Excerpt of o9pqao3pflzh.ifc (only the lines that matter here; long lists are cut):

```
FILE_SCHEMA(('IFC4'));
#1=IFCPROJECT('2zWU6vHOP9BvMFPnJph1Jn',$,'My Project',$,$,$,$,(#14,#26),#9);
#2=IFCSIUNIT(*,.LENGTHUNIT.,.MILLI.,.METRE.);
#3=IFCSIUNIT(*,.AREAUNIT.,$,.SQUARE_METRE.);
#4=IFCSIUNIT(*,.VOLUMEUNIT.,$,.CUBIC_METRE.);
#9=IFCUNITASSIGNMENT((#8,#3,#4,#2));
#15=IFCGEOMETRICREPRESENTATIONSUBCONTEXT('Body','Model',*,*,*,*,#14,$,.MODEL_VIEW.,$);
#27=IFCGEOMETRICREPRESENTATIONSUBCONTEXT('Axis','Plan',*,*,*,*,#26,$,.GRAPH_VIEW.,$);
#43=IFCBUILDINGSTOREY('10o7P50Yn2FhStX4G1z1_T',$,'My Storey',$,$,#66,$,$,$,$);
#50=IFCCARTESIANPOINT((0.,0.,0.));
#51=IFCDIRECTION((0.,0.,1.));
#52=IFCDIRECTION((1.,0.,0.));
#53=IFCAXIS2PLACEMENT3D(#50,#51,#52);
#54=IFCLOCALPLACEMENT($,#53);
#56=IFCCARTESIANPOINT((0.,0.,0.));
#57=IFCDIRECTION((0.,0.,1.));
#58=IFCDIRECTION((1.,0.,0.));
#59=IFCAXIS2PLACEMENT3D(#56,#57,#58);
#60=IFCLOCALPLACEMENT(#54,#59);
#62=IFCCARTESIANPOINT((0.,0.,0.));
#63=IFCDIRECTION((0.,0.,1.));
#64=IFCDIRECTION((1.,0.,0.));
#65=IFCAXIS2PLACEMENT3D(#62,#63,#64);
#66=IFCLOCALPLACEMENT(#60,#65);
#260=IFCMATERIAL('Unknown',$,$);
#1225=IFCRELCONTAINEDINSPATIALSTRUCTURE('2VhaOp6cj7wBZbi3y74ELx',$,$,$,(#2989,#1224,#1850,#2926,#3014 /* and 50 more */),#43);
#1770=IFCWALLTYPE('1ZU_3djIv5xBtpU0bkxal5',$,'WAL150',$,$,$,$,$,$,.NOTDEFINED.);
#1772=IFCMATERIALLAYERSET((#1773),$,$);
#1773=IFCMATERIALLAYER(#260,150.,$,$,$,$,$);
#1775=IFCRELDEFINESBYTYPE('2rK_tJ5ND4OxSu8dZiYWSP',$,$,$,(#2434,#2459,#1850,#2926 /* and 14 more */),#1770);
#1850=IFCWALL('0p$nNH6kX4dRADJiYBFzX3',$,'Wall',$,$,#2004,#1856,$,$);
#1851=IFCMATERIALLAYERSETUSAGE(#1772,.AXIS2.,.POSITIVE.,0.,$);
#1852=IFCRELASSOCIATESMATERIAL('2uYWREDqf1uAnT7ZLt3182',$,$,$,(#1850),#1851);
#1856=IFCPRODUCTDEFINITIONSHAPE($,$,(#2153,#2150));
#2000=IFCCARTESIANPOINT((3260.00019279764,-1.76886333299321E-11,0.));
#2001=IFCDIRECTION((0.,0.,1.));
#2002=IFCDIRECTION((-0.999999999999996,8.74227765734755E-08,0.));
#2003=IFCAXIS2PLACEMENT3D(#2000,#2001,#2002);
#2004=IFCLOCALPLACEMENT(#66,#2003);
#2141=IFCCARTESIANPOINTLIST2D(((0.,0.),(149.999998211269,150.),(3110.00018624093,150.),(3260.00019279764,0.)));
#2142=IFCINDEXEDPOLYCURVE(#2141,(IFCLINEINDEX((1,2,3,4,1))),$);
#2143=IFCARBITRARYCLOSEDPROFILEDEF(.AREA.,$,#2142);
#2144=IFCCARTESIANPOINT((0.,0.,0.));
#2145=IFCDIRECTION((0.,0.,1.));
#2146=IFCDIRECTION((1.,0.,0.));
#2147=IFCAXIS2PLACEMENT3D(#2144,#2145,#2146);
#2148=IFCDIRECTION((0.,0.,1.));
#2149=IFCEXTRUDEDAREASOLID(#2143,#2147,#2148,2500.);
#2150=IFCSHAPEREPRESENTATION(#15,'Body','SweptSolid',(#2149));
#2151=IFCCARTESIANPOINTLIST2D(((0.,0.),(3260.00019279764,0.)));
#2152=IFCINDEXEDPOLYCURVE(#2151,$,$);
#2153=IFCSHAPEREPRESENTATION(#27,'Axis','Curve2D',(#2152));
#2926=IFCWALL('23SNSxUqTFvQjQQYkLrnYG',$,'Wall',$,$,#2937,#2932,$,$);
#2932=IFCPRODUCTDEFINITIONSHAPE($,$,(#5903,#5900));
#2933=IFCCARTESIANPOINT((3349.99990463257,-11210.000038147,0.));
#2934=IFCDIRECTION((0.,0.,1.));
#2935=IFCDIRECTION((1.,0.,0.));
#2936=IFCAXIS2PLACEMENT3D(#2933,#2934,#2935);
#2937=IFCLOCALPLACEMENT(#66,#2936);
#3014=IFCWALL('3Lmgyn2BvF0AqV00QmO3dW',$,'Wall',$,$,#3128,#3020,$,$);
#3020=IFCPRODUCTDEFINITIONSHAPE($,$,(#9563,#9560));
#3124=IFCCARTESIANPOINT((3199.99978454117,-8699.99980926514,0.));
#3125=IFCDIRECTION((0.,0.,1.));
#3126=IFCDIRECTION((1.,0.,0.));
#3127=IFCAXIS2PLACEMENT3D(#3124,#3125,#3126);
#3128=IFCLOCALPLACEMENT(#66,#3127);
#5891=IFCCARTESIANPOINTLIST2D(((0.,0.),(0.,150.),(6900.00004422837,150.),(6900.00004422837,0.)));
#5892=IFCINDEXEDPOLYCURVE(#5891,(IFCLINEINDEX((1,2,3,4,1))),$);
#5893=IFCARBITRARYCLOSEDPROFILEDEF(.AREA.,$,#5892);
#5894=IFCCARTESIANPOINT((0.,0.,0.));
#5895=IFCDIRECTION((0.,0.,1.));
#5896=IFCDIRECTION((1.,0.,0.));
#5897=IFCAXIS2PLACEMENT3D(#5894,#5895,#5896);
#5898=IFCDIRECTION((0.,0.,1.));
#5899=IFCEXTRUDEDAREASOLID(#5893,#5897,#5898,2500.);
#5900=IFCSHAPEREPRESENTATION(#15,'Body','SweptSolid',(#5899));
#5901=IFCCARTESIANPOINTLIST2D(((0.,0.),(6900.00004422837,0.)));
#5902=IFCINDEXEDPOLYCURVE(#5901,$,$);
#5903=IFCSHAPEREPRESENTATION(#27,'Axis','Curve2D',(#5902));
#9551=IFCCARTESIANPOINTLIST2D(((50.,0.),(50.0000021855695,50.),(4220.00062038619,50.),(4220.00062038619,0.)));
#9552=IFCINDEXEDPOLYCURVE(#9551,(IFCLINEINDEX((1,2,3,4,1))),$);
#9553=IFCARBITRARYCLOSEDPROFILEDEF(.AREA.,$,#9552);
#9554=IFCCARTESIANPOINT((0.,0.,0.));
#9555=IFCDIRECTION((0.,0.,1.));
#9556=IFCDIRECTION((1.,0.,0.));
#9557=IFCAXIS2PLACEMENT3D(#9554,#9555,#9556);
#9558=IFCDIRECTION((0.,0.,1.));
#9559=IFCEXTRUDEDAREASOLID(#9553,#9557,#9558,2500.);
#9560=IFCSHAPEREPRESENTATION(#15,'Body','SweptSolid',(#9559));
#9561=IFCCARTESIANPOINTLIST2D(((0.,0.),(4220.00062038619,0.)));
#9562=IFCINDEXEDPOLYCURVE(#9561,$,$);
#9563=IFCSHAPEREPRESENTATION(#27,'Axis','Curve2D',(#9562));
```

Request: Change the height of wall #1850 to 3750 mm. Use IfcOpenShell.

```python
import ifcopenshell
import ifcopenshell.geom
import ifcopenshell.util.representation
import ifcopenshell.util.shape

model = ifcopenshell.open("o9pqao3pflzh.ifc")
settings = ifcopenshell.geom.settings()


def volume(element):
    """Net volume in cubic metres, openings subtracted."""
    shape = ifcopenshell.geom.create_shape(settings, element)
    return ifcopenshell.util.shape.get_volume(shape.geometry)


wall = model.by_id(1850)
before = volume(wall)

body = ifcopenshell.util.representation.get_representation(wall, "Model", "Body")
solid = body.Items[0]
old_height = solid.Depth
solid.Depth = 3750.0
after = volume(wall)

print(f"height {old_height:g} -> {solid.Depth:g}, volume {before:.3f} -> {after:.3f} m3")

model.write("o9pqao3pflzh-out.ifc")
```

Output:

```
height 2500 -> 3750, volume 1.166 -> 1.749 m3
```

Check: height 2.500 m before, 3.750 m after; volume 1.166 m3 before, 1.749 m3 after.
